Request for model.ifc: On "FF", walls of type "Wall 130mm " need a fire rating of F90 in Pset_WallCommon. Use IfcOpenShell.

First a look at what the model holds.

```python
import ifcopenshell
import ifcopenshell.util.element

model = ifcopenshell.open("model.ifc")
print(model.schema)
storey = next(s for s in model.by_type("IfcBuildingStorey") if s.Name == "FF")
walls = [e for e in ifcopenshell.util.element.get_decomposition(storey) if e.is_a("IfcWall")]
seen = {}
for e in walls:
    element_type = ifcopenshell.util.element.get_type(e)
    key = (element_type.Name if element_type != e and element_type else None, ifcopenshell.util.element.get_pset(e, "Pset_WallCommon", "FireRating"))
    seen[key] = seen.get(key, 0) + 1
for (name, value), count in sorted(seen.items(), key=str):
    print(count, "x", name, "|", value)
```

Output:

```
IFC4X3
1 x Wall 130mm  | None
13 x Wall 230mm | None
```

```python
import ifcopenshell
import ifcopenshell.api.pset
import ifcopenshell.util.element

model = ifcopenshell.open("model.ifc")

storey = next(s for s in model.by_type("IfcBuildingStorey") if s.Name == "FF")
walls = [e for e in ifcopenshell.util.element.get_decomposition(storey) if e.is_a("IfcWall")]

count = 0
for e in walls:
    element_type = ifcopenshell.util.element.get_type(e)
    if element_type in (None, e) or element_type.Name != "Wall 130mm ":
        continue
    # add_pset returns the element's existing set when there is one.
    pset = ifcopenshell.api.pset.add_pset(model, product=e, name="Pset_WallCommon")
    ifcopenshell.api.pset.edit_pset(model, pset=pset, properties={"FireRating": "F90"})
    count += 1

print(count, "walls updated")

model.write("model_rev.ifc")
```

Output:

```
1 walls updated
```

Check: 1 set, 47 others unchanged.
